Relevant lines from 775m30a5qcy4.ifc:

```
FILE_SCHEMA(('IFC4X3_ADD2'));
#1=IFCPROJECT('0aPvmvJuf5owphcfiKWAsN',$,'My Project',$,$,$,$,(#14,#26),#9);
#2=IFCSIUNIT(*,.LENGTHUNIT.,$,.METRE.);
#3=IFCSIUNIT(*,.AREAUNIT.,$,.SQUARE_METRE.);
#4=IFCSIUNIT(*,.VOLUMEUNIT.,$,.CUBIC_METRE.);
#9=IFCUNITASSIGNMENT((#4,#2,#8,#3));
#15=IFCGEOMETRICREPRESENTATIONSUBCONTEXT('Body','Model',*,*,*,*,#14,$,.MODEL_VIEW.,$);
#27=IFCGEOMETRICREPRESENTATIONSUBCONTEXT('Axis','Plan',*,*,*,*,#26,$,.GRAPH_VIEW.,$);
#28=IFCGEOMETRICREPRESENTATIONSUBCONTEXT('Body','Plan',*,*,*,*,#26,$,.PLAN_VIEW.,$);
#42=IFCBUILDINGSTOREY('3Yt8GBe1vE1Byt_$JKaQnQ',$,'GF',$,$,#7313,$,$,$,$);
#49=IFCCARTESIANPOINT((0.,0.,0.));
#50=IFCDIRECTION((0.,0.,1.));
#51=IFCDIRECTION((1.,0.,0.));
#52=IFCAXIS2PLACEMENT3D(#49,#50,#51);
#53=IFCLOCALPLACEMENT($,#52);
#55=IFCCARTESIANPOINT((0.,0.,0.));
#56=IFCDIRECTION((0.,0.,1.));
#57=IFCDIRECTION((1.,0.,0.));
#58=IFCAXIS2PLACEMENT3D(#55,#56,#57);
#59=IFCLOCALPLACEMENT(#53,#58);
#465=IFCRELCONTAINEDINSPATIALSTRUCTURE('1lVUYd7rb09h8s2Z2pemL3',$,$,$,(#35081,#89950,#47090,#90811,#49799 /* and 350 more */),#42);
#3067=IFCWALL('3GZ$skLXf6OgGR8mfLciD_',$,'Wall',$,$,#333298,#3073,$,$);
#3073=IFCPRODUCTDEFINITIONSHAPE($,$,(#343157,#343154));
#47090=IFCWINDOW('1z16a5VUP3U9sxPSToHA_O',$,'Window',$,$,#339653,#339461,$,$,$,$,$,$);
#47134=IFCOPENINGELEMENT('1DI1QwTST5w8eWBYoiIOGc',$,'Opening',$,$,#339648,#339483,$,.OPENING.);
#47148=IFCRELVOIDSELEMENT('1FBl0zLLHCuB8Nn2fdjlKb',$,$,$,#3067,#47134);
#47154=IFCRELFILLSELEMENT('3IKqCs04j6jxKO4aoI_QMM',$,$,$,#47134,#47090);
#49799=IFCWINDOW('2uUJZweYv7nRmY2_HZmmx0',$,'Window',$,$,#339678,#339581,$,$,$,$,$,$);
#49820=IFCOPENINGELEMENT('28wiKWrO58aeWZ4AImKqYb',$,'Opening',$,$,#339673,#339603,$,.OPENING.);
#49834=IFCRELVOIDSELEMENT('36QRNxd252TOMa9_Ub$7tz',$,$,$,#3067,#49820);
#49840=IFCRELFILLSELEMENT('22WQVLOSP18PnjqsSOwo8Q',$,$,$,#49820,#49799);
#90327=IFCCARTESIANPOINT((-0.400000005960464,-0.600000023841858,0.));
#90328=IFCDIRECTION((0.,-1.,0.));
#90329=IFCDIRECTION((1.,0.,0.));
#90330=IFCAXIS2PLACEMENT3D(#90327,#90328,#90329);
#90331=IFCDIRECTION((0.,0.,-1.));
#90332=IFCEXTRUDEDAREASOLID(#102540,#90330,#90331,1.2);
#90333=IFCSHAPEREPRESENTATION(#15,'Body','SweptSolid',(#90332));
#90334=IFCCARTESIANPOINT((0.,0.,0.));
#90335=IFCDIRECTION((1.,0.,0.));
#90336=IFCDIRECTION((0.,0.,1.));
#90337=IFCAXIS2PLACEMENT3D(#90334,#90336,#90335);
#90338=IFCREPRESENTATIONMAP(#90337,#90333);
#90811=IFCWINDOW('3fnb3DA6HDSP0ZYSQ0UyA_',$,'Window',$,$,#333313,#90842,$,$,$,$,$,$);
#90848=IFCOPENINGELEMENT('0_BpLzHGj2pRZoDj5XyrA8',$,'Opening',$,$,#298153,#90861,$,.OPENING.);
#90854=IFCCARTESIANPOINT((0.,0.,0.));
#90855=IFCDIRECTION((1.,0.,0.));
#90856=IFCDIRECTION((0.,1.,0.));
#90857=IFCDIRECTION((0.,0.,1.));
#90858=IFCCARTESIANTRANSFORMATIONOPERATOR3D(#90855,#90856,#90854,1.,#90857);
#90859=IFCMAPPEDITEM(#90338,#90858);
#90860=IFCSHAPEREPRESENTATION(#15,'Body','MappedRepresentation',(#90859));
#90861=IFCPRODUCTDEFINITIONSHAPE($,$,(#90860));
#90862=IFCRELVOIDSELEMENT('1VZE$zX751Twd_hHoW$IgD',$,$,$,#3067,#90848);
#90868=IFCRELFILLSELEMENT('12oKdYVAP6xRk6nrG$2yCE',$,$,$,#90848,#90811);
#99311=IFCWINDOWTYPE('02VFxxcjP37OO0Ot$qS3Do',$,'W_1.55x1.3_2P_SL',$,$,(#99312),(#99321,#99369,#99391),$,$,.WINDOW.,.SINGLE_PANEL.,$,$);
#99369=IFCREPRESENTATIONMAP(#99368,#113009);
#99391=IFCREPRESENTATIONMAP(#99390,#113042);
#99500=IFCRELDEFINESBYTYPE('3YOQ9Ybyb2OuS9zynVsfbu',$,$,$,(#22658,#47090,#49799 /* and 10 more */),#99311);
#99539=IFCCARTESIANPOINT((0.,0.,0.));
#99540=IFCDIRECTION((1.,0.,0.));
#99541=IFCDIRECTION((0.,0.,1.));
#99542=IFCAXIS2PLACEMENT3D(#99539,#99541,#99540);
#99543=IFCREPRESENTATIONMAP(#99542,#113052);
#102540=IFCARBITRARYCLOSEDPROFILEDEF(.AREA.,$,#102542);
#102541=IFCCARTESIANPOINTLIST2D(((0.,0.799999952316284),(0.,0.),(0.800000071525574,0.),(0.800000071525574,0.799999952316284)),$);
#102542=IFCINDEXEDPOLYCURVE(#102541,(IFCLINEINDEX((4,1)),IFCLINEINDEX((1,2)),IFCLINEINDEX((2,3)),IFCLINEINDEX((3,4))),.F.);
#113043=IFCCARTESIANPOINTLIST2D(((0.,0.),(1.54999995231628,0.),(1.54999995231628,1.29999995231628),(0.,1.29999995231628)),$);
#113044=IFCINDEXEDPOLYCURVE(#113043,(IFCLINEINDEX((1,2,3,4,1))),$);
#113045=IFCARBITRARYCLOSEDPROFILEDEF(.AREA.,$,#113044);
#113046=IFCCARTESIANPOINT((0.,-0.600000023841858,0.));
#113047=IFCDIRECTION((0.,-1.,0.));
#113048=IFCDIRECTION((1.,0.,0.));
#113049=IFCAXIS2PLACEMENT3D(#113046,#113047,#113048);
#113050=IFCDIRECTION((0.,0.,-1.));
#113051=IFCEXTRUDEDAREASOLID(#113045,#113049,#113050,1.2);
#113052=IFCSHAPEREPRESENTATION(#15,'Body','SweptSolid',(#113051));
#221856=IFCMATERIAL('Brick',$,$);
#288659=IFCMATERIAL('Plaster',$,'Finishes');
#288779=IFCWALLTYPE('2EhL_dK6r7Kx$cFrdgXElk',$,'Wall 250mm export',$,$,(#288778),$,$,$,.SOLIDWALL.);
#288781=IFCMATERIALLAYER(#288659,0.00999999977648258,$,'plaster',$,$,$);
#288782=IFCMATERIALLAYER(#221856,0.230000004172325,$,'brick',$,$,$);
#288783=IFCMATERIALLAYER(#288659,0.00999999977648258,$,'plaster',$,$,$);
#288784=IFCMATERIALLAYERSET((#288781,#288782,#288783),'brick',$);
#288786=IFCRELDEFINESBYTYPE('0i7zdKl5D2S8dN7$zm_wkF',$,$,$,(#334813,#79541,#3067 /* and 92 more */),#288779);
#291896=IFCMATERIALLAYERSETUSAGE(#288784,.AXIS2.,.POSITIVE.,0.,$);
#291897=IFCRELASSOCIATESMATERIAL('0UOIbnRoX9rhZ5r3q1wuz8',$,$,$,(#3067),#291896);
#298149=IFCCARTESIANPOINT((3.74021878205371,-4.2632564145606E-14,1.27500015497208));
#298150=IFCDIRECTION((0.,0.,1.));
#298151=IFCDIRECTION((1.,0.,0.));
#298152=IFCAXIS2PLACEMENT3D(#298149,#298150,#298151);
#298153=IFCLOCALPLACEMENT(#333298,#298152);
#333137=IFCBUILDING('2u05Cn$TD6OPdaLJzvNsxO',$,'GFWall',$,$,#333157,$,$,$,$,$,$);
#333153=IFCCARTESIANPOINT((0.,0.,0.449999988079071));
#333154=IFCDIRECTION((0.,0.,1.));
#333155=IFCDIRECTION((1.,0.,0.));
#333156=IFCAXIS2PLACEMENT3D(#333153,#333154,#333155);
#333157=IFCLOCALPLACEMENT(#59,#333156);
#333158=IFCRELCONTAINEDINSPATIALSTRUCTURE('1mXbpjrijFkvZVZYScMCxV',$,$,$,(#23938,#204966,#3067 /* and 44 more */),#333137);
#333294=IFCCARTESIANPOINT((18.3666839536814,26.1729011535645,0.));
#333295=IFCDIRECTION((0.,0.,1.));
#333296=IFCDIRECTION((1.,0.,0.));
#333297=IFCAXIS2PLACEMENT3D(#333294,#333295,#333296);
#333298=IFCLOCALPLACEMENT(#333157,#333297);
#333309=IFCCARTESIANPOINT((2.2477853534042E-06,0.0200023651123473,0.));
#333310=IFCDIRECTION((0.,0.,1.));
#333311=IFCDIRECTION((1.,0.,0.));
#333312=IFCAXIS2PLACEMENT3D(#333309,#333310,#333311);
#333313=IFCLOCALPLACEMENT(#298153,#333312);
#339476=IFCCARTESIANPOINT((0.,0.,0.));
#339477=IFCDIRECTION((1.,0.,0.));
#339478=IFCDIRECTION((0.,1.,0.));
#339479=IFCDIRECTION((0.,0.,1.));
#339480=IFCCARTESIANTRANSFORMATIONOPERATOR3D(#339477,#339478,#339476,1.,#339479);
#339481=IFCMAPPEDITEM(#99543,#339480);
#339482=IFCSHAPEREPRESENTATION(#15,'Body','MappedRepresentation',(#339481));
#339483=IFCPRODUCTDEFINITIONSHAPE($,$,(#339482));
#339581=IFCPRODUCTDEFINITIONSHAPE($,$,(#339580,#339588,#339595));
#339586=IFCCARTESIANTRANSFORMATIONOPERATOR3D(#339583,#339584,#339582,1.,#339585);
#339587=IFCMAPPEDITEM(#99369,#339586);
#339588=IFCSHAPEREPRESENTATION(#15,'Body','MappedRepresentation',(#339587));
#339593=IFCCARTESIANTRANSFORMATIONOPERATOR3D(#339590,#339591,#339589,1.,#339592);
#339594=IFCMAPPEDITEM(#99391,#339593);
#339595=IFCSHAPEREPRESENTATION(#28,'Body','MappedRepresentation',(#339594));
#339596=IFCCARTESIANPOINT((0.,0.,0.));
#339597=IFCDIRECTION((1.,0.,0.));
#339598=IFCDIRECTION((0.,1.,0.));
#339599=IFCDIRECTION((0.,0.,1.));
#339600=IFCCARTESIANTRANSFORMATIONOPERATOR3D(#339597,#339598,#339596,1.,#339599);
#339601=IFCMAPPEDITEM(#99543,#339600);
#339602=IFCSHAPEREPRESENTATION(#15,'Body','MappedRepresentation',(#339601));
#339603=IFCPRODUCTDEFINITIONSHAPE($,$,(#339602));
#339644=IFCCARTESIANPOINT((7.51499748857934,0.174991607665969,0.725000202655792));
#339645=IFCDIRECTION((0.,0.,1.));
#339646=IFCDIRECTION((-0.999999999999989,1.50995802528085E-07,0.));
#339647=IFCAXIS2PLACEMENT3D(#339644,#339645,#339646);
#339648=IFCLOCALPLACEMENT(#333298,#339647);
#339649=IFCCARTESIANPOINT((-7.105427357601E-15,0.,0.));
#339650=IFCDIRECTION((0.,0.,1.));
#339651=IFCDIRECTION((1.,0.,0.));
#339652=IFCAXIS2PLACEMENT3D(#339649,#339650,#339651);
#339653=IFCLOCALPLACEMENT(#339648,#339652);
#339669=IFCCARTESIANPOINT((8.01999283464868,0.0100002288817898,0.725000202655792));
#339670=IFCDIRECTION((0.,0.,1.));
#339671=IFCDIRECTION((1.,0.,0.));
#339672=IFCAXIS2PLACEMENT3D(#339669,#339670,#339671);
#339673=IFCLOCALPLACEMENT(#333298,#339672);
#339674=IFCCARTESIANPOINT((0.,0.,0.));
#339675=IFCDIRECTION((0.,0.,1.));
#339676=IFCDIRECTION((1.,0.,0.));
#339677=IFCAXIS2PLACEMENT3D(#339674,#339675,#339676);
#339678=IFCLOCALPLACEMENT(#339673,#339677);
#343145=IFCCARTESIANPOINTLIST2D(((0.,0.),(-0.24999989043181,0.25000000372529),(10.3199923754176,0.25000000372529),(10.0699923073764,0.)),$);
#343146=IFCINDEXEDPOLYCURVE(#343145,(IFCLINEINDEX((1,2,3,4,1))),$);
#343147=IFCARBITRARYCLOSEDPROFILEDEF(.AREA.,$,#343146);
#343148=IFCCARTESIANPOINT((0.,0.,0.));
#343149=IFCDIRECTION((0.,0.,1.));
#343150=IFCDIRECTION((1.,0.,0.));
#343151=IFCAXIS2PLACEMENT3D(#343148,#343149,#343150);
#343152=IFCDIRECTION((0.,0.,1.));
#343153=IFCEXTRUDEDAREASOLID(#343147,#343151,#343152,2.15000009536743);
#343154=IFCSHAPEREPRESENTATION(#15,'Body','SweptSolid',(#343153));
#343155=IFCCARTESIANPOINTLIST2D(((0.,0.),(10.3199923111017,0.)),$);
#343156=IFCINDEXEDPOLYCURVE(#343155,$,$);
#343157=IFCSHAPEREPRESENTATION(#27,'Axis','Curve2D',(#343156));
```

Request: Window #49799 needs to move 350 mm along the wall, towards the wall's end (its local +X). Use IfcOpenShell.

```python
import ifcopenshell
import ifcopenshell.api.geometry
import ifcopenshell.util.placement

model = ifcopenshell.open("775m30a5qcy4.ifc")

window = model.by_guid("2uUJZweYv7nRmY2_HZmmx0")
opening = window.FillsVoids[0].RelatingOpeningElement
wall = opening.VoidsElements[0].RelatingBuildingElement

wall_matrix = ifcopenshell.util.placement.get_local_placement(wall.ObjectPlacement)
shift = wall_matrix[:3, 0] * 0.35
before = ifcopenshell.util.placement.get_local_placement(window.ObjectPlacement)[:3, 3].copy()

# The window is placed relative to its opening, so it follows when the opening moves.
matrix = ifcopenshell.util.placement.get_local_placement(opening.ObjectPlacement)
matrix[:3, 3] += shift
ifcopenshell.api.geometry.edit_object_placement(
    model, product=opening, matrix=matrix, is_si=False, should_transform_children=True
)

after = ifcopenshell.util.placement.get_local_placement(window.ObjectPlacement)[:3, 3]
print("window moved by", (after - before).round(3) + 0.0)

model.write("775m30a5qcy4_rev.ifc")
```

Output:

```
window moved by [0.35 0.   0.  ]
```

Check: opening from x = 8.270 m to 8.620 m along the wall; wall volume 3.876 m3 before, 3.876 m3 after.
